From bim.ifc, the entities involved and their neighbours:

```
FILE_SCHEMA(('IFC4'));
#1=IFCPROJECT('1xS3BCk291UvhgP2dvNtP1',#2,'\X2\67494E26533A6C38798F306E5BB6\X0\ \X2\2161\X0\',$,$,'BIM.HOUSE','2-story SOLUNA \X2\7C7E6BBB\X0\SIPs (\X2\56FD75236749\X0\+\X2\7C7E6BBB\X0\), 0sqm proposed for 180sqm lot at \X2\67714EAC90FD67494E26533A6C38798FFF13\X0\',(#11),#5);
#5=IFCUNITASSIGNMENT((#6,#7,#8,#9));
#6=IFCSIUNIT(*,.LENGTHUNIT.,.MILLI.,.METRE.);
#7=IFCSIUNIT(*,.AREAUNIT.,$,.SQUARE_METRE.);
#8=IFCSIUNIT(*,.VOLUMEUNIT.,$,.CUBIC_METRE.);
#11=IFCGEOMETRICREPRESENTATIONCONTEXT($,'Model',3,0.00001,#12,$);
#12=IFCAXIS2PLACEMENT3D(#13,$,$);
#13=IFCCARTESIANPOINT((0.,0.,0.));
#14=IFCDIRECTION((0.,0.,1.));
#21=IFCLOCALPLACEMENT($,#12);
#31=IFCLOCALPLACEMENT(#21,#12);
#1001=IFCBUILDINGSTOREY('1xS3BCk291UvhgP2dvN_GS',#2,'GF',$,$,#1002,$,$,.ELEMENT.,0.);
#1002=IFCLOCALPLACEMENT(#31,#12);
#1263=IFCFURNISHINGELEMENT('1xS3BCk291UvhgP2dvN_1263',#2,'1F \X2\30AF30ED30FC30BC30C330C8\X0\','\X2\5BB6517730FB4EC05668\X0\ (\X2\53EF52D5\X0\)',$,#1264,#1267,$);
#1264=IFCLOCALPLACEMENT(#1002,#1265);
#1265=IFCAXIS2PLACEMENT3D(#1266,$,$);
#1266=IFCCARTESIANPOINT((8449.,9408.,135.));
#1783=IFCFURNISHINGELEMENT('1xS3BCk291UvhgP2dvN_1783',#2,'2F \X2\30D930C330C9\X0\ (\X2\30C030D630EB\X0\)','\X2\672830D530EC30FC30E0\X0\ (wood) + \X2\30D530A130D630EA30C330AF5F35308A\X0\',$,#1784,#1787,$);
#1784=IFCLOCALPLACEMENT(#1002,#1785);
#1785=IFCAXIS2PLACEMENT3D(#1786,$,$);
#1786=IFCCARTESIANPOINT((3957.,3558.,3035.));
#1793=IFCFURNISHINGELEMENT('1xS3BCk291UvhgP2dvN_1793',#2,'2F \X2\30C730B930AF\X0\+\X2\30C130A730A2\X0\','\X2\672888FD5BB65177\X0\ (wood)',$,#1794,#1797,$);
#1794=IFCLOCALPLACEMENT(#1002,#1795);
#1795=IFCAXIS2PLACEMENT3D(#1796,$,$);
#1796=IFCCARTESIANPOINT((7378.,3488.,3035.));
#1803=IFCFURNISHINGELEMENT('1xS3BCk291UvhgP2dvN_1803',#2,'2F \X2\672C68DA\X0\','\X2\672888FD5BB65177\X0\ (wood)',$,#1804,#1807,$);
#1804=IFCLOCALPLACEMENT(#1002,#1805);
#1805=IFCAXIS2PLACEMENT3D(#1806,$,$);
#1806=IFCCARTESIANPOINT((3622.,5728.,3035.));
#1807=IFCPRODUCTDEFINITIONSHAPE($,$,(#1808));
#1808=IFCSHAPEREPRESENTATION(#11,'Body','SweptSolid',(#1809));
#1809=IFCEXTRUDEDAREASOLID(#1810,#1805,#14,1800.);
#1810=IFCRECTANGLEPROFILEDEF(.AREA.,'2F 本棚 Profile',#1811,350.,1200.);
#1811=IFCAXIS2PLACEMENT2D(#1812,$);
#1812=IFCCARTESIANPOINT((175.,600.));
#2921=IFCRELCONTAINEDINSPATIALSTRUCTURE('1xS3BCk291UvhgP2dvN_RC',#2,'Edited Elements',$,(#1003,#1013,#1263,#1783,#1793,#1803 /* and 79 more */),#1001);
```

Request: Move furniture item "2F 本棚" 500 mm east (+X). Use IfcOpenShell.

```python
import ifcopenshell
import ifcopenshell.api.geometry
import ifcopenshell.util.placement

model = ifcopenshell.open("bim.ifc")

item = model.by_guid("1xS3BCk291UvhgP2dvN_1803")
matrix = ifcopenshell.util.placement.get_local_placement(item.ObjectPlacement)
matrix[0, 3] += 500.0
ifcopenshell.api.geometry.edit_object_placement(model, product=item, matrix=matrix, is_si=False)

print(ifcopenshell.util.placement.get_local_placement(item.ObjectPlacement).round(3) + 0.0)

model.write("bim_rev.ifc")
```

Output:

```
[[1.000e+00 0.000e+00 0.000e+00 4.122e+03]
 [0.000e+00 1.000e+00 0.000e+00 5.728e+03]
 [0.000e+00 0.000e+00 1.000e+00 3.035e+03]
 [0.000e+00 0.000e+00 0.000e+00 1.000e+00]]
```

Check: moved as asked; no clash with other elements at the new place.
